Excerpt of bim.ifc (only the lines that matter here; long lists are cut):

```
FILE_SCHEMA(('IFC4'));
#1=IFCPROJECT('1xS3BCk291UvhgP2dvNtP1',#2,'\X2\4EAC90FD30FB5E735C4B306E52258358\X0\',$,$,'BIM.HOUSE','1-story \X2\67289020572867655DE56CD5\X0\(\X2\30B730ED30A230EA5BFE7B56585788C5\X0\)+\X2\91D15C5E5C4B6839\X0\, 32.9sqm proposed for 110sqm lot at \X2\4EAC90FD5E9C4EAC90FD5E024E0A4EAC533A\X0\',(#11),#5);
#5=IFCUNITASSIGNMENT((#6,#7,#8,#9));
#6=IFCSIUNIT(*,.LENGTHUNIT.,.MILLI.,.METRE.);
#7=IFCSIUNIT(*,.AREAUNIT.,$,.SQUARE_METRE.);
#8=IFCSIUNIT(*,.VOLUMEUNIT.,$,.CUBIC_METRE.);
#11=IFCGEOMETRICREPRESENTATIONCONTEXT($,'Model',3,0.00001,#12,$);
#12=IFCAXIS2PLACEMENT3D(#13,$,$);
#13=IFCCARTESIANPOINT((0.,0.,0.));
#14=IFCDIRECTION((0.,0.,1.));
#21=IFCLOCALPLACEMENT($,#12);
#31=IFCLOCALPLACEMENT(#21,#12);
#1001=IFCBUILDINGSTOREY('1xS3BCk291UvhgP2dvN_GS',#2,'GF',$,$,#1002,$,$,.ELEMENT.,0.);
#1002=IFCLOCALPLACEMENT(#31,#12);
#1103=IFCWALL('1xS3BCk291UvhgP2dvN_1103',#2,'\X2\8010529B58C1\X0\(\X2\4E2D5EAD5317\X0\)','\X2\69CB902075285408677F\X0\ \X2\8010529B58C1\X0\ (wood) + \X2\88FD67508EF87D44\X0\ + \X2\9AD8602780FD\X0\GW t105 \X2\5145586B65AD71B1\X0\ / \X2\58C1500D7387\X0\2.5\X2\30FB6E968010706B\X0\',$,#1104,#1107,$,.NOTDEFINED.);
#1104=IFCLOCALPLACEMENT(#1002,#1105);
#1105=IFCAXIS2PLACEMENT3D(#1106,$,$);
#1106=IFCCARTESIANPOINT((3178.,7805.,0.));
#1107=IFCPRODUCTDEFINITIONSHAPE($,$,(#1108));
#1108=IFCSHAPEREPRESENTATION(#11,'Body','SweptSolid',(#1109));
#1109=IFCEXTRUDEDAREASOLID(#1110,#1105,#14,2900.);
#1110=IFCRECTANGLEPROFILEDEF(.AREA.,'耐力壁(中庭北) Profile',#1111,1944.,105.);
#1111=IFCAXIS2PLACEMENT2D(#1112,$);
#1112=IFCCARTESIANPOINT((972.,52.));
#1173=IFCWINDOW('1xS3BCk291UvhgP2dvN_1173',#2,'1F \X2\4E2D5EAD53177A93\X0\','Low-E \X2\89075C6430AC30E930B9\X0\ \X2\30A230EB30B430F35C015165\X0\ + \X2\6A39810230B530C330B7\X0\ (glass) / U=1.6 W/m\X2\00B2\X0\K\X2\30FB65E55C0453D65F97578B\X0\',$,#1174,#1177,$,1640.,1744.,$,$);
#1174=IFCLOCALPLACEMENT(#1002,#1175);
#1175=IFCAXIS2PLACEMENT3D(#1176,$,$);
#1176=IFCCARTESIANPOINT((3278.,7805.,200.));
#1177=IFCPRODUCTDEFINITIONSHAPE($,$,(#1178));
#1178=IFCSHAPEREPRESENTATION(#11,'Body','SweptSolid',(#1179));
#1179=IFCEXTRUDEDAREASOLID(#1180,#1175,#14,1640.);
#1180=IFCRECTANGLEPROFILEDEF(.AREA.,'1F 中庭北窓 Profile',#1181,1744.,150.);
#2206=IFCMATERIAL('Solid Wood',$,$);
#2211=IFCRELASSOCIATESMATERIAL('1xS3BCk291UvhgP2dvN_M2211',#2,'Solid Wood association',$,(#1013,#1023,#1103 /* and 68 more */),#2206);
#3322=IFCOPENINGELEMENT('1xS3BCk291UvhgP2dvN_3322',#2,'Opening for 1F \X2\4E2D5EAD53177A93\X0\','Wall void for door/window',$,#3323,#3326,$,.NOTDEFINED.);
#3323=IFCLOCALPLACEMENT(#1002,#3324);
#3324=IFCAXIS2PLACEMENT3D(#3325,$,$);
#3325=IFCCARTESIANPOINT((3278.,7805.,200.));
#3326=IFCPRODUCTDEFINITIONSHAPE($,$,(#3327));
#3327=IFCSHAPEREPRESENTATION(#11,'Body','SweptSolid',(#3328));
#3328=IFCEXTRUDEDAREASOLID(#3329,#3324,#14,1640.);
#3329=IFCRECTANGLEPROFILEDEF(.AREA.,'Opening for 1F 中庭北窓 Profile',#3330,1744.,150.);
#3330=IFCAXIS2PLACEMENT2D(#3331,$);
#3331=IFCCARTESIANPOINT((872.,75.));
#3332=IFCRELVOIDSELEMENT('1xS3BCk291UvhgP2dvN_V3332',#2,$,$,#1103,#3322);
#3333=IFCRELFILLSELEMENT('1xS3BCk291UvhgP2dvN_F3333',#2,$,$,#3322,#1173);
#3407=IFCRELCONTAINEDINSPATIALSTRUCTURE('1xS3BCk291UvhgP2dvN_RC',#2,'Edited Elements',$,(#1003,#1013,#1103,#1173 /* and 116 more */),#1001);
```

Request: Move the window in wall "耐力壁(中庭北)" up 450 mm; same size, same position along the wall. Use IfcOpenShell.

```python
import numpy as np
import ifcopenshell
import ifcopenshell.api.geometry
import ifcopenshell.util.placement
import ifcopenshell.util.unit

model = ifcopenshell.open("bim.ifc")
unit_scale = ifcopenshell.util.unit.calculate_unit_scale(model)

window = model.by_id(1173)
opening = window.FillsVoids[0].RelatingOpeningElement
dz = 450.0

shift = np.array([0.0, 0.0, dz])
# The window is not placed relative to its opening, so move both.
for product in (opening, window):
    matrix = ifcopenshell.util.placement.get_local_placement(product.ObjectPlacement)
    matrix[:3, 3] += shift
    ifcopenshell.api.geometry.edit_object_placement(model, product=product, matrix=matrix, is_si=False)

print(f"moved by {dz * unit_scale:+.3f} m")

model.write("bim_rev.ifc")
```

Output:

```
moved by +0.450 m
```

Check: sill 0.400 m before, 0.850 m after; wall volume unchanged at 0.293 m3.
